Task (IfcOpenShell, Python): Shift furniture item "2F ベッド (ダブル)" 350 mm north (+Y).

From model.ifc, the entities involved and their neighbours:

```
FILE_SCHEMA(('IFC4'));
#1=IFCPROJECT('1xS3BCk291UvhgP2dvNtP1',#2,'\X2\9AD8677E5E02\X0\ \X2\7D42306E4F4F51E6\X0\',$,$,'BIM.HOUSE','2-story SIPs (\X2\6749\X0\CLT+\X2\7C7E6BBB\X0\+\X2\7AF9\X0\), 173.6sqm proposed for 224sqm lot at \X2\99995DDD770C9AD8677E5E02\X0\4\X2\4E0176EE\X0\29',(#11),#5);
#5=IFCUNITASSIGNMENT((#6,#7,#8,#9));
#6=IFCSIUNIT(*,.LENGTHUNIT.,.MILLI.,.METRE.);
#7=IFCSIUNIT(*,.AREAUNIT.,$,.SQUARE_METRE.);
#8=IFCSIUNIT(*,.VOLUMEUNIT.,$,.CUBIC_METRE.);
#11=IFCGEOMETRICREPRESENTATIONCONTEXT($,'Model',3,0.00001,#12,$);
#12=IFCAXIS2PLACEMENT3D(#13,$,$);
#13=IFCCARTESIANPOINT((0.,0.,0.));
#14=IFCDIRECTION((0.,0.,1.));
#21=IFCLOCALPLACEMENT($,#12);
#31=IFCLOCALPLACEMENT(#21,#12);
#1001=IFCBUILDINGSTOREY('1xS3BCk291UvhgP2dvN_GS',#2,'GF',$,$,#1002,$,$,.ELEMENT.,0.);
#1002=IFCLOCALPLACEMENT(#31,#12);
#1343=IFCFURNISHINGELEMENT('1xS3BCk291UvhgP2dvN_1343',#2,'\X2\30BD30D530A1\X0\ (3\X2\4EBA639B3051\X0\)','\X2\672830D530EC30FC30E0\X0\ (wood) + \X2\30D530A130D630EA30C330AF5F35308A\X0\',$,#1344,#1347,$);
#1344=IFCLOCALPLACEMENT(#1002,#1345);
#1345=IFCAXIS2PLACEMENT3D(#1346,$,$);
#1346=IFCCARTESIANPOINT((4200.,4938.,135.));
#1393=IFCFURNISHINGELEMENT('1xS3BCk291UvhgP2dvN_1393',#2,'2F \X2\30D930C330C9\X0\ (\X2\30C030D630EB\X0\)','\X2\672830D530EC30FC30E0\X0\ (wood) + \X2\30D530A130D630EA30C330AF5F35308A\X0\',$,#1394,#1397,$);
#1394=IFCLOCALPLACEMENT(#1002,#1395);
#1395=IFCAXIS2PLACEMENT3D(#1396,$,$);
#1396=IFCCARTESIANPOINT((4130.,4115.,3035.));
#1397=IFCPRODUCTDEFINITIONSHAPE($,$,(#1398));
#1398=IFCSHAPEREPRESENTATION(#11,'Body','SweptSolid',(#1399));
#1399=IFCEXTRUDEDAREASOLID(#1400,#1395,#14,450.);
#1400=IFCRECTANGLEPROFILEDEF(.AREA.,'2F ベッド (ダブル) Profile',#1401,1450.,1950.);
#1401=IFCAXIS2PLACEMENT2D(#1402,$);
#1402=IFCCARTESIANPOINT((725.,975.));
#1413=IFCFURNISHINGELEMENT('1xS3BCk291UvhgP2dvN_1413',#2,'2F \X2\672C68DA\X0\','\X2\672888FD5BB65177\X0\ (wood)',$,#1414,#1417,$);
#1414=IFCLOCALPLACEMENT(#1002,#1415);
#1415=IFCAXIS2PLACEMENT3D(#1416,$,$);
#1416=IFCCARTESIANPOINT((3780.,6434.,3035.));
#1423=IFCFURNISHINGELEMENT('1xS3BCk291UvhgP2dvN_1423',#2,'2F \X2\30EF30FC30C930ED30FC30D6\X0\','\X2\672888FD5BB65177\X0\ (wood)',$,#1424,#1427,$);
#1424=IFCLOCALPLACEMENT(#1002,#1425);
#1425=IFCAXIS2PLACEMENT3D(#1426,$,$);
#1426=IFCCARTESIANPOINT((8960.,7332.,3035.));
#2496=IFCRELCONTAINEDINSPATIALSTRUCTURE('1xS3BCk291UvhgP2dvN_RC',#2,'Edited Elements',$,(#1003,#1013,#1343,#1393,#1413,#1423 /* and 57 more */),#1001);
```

```python
import ifcopenshell
import ifcopenshell.api.geometry
import ifcopenshell.util.placement

model = ifcopenshell.open("model.ifc")

item = model.by_guid("1xS3BCk291UvhgP2dvN_1393")
matrix = ifcopenshell.util.placement.get_local_placement(item.ObjectPlacement)
matrix[1, 3] += 350.0
ifcopenshell.api.geometry.edit_object_placement(model, product=item, matrix=matrix, is_si=False)

print(ifcopenshell.util.placement.get_local_placement(item.ObjectPlacement).round(3) + 0.0)

model.write("model_edited.ifc")
```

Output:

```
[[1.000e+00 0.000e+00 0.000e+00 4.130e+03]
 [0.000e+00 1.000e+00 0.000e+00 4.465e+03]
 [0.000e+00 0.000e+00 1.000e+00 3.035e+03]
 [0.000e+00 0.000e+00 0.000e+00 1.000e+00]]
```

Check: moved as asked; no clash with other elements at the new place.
